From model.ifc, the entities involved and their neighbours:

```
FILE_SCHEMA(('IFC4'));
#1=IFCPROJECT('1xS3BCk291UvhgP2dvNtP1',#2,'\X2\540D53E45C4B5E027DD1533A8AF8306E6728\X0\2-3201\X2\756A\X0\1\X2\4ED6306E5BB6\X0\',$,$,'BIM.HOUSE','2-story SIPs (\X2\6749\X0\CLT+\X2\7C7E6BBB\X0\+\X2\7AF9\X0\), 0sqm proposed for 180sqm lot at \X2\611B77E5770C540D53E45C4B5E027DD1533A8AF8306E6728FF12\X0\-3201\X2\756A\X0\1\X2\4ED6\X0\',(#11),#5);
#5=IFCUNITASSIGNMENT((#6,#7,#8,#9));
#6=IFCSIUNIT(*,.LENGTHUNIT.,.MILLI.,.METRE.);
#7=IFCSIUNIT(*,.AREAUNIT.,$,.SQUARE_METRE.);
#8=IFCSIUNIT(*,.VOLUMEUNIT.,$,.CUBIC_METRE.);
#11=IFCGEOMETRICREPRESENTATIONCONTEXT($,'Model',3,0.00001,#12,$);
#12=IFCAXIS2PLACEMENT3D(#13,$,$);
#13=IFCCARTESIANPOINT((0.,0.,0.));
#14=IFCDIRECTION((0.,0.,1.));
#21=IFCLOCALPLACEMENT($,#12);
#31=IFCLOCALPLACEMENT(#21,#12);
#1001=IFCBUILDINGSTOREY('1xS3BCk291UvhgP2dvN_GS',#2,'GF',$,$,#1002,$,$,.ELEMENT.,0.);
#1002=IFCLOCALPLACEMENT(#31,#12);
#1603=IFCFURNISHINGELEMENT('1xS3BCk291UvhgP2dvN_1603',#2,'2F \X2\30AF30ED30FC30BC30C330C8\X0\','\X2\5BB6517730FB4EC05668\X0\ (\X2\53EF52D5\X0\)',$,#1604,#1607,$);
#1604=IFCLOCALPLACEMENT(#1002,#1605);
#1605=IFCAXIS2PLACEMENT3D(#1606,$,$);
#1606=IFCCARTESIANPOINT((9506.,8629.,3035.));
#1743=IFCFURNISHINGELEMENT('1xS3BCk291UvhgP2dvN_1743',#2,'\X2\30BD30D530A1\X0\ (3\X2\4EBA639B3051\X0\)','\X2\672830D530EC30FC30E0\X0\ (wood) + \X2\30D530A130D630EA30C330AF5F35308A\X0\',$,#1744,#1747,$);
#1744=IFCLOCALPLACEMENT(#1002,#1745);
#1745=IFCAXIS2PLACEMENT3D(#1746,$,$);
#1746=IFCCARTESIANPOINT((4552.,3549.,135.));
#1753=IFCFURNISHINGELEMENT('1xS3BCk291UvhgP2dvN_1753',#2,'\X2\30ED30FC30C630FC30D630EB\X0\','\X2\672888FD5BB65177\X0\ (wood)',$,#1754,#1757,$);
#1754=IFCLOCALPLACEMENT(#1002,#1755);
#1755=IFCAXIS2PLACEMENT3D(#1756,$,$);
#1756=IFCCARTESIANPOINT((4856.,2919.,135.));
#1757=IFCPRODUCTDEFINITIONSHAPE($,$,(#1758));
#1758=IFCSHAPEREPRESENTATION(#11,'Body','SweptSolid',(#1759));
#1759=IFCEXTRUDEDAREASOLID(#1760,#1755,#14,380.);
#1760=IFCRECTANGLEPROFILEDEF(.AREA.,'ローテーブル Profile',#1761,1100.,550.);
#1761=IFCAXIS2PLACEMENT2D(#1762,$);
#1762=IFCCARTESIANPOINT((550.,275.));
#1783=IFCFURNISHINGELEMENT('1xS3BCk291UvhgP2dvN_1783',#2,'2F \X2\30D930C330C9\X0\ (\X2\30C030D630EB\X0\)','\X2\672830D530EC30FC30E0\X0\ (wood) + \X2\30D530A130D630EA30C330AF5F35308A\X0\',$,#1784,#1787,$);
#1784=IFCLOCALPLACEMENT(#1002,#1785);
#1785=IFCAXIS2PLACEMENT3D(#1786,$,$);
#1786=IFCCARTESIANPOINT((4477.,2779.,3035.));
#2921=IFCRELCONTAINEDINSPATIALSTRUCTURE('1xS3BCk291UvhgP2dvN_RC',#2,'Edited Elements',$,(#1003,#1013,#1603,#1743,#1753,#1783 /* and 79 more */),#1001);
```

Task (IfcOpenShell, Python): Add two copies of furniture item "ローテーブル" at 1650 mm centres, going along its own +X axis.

```python
import ifcopenshell
import ifcopenshell.api.geometry
import ifcopenshell.api.root
import ifcopenshell.util.element
import ifcopenshell.util.placement
import ifcopenshell.util.unit

model = ifcopenshell.open("model.ifc")
unit_scale = ifcopenshell.util.unit.calculate_unit_scale(model)


def reuse_history(source, copy):
    """copy_class also copies each property set's owner history, people and application; keep the originals."""
    for rel in copy.IsDefinedBy:
        if rel.is_a("IfcRelDefinesByProperties") and (history := rel.RelatingPropertyDefinition.OwnerHistory):
            rel.RelatingPropertyDefinition.OwnerHistory = source.OwnerHistory
            ifcopenshell.util.element.remove_deep2(model, history)


source = model.by_id(1753)
base = ifcopenshell.util.placement.get_local_placement(source.ObjectPlacement)
step = base[:3, 0] * 1.65 / unit_scale

for i in range(1, 3):
    copy = ifcopenshell.api.root.copy_class(model, product=source)
    copy.Representation = ifcopenshell.util.element.copy_deep(
        model, source.Representation, exclude=["IfcGeometricRepresentationContext", "IfcRepresentationMap"]
    )
    reuse_history(source, copy)
    matrix = base.copy()
    matrix[:3, 3] += i * step
    print("added at", matrix[:3, 3].round(3) + 0.0)
    ifcopenshell.api.geometry.edit_object_placement(model, product=copy, matrix=matrix, is_si=False)

model.write("model_rev.ifc")
```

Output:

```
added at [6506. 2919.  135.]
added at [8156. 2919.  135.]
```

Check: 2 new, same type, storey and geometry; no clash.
